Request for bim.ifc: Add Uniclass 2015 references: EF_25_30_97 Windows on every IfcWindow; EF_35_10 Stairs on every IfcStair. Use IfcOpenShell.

First a look at what the model holds.

```python
import ifcopenshell

model = ifcopenshell.open("bim.ifc")
print(model.schema)
print("classifications:", [c.Name for c in model.by_type("IfcClassification")])
for ifc_class in ("IfcDoor", "IfcRoof", "IfcStair", "IfcWall", "IfcWindow"):
    print(ifc_class, len(model.by_type(ifc_class)))
```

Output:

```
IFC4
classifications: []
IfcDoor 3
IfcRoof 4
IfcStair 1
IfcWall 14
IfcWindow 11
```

```python
import ifcopenshell
import ifcopenshell.api.classification

model = ifcopenshell.open("bim.ifc")

system = ifcopenshell.api.classification.add_classification(model, classification="Uniclass 2015")

codes = {
    "IfcWindow": ("EF_25_30_97", "Windows"),
    "IfcStair": ("EF_35_10", "Stairs"),
}
for ifc_class, (code, name) in codes.items():
    products = model.by_type(ifc_class)
    ifcopenshell.api.classification.add_reference(
        model, products=products, classification=system, identification=code, name=name
    )
    print(code, len(products))

model.write("bim-out.ifc")
```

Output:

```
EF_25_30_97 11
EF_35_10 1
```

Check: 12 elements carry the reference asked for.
